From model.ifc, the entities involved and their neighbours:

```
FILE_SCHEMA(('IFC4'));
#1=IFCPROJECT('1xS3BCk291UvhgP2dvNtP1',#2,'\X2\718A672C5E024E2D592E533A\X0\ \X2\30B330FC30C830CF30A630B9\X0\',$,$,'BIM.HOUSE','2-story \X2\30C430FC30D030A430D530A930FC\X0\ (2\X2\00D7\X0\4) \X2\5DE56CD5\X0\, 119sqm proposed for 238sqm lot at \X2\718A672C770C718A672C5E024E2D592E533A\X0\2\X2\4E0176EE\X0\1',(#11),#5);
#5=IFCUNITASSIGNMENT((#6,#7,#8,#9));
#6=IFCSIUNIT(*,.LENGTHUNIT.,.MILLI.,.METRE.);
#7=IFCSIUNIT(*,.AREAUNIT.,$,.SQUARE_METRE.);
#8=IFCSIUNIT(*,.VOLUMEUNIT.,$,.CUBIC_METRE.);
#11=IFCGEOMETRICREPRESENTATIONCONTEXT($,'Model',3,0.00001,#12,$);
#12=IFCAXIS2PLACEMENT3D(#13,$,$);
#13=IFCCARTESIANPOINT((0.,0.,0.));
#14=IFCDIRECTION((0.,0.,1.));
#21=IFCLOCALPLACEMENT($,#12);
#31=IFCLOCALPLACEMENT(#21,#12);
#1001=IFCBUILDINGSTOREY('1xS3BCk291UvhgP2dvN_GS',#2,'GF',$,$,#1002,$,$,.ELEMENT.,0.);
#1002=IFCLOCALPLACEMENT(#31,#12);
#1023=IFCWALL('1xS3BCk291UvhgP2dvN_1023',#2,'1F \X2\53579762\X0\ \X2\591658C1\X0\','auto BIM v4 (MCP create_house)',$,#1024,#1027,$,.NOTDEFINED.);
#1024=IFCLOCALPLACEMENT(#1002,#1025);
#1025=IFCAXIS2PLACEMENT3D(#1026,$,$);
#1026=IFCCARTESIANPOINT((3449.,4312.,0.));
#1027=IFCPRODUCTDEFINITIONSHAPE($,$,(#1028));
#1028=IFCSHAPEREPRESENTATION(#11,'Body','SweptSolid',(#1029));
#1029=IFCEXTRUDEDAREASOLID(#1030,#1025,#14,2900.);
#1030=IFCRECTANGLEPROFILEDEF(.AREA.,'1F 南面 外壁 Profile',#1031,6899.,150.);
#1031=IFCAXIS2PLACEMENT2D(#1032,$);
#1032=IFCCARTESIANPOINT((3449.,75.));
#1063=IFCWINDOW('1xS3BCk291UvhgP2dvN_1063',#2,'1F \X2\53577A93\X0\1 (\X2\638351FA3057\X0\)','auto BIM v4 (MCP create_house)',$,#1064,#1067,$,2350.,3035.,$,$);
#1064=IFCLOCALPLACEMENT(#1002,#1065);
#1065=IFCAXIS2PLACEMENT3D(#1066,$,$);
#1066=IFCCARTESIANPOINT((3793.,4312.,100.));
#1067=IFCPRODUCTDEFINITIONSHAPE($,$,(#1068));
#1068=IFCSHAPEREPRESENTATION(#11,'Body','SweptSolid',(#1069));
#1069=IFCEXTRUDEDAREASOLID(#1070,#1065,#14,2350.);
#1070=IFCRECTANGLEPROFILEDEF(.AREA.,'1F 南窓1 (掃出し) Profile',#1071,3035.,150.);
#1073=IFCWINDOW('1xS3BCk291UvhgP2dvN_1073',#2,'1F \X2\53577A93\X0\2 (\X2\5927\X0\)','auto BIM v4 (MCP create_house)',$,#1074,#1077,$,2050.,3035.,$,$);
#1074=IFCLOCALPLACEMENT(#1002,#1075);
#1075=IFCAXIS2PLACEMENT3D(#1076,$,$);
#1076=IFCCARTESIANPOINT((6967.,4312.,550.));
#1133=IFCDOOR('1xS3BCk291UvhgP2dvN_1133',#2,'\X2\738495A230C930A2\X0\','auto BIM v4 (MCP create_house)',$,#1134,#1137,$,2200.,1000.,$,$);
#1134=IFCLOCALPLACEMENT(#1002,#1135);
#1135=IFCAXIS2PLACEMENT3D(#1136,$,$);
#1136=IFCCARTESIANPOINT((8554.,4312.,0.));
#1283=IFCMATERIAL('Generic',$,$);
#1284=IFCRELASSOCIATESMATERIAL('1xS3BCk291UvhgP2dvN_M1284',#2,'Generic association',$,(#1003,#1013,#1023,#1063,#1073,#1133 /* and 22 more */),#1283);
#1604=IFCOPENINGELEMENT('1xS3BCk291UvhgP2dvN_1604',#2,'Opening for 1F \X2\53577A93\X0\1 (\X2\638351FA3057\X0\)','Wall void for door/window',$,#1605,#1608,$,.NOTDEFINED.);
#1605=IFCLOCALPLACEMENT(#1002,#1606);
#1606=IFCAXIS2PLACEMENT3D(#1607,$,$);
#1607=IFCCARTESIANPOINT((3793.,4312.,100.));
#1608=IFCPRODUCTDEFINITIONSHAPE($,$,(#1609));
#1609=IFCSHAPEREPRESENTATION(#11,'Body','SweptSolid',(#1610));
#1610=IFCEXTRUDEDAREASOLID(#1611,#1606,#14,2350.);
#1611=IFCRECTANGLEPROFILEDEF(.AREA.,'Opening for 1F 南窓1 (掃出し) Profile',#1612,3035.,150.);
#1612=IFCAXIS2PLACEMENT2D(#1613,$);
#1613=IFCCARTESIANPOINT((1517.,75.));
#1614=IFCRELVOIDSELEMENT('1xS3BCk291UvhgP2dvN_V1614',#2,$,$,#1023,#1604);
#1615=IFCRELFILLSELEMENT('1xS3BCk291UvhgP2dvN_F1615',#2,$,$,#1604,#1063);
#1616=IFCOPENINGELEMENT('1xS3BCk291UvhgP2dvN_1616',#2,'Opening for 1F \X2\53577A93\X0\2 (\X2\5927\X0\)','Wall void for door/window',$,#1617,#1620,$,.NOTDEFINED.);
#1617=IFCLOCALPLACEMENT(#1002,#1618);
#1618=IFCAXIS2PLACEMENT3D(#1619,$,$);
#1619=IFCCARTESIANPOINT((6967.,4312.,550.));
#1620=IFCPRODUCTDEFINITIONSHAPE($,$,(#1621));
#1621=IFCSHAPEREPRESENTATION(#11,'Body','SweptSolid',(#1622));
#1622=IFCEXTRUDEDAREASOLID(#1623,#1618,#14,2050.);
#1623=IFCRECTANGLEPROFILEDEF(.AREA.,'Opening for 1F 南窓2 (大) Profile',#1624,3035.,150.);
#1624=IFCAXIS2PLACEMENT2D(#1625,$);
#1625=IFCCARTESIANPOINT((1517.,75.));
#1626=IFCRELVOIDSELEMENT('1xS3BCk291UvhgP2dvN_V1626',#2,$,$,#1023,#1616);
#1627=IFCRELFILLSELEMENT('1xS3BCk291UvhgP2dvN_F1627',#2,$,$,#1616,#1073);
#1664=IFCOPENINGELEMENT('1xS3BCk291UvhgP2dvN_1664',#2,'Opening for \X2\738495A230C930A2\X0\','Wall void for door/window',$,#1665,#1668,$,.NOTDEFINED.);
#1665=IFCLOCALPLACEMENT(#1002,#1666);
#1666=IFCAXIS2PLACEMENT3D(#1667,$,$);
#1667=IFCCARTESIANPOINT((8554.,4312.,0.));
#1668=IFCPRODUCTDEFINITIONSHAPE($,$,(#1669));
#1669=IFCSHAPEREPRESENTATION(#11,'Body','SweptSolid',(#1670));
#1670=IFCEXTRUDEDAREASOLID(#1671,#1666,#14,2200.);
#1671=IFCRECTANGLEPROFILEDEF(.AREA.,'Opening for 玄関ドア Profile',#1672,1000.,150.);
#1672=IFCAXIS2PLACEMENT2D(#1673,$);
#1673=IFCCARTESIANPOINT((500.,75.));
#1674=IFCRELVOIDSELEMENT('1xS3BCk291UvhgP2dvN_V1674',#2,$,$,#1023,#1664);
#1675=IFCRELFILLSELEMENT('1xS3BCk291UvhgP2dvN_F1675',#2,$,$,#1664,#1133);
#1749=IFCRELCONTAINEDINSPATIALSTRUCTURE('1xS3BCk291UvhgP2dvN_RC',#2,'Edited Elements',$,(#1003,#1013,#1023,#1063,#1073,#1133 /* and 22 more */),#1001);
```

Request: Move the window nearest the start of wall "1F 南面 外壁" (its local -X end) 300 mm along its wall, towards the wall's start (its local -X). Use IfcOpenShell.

```python
import ifcopenshell
import ifcopenshell.api.geometry
import ifcopenshell.util.placement
import ifcopenshell.util.unit

model = ifcopenshell.open("model.ifc")
unit_scale = ifcopenshell.util.unit.calculate_unit_scale(model)

window = model.by_guid("1xS3BCk291UvhgP2dvN_1063")
opening = window.FillsVoids[0].RelatingOpeningElement
wall = opening.VoidsElements[0].RelatingBuildingElement

wall_matrix = ifcopenshell.util.placement.get_local_placement(wall.ObjectPlacement)
shift = wall_matrix[:3, 0] * -0.3 / unit_scale
before = ifcopenshell.util.placement.get_local_placement(window.ObjectPlacement)[:3, 3].copy()

# The window is not placed relative to its opening, so move both.
for product in (opening, window):
    matrix = ifcopenshell.util.placement.get_local_placement(product.ObjectPlacement)
    matrix[:3, 3] += shift
    ifcopenshell.api.geometry.edit_object_placement(model, product=product, matrix=matrix, is_si=False)

after = ifcopenshell.util.placement.get_local_placement(window.ObjectPlacement)[:3, 3]
print("window moved by", (after - before).round(3) + 0.0)

model.write("model_edited.ifc")
```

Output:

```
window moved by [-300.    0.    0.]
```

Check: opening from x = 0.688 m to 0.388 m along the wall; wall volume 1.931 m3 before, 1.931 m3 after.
